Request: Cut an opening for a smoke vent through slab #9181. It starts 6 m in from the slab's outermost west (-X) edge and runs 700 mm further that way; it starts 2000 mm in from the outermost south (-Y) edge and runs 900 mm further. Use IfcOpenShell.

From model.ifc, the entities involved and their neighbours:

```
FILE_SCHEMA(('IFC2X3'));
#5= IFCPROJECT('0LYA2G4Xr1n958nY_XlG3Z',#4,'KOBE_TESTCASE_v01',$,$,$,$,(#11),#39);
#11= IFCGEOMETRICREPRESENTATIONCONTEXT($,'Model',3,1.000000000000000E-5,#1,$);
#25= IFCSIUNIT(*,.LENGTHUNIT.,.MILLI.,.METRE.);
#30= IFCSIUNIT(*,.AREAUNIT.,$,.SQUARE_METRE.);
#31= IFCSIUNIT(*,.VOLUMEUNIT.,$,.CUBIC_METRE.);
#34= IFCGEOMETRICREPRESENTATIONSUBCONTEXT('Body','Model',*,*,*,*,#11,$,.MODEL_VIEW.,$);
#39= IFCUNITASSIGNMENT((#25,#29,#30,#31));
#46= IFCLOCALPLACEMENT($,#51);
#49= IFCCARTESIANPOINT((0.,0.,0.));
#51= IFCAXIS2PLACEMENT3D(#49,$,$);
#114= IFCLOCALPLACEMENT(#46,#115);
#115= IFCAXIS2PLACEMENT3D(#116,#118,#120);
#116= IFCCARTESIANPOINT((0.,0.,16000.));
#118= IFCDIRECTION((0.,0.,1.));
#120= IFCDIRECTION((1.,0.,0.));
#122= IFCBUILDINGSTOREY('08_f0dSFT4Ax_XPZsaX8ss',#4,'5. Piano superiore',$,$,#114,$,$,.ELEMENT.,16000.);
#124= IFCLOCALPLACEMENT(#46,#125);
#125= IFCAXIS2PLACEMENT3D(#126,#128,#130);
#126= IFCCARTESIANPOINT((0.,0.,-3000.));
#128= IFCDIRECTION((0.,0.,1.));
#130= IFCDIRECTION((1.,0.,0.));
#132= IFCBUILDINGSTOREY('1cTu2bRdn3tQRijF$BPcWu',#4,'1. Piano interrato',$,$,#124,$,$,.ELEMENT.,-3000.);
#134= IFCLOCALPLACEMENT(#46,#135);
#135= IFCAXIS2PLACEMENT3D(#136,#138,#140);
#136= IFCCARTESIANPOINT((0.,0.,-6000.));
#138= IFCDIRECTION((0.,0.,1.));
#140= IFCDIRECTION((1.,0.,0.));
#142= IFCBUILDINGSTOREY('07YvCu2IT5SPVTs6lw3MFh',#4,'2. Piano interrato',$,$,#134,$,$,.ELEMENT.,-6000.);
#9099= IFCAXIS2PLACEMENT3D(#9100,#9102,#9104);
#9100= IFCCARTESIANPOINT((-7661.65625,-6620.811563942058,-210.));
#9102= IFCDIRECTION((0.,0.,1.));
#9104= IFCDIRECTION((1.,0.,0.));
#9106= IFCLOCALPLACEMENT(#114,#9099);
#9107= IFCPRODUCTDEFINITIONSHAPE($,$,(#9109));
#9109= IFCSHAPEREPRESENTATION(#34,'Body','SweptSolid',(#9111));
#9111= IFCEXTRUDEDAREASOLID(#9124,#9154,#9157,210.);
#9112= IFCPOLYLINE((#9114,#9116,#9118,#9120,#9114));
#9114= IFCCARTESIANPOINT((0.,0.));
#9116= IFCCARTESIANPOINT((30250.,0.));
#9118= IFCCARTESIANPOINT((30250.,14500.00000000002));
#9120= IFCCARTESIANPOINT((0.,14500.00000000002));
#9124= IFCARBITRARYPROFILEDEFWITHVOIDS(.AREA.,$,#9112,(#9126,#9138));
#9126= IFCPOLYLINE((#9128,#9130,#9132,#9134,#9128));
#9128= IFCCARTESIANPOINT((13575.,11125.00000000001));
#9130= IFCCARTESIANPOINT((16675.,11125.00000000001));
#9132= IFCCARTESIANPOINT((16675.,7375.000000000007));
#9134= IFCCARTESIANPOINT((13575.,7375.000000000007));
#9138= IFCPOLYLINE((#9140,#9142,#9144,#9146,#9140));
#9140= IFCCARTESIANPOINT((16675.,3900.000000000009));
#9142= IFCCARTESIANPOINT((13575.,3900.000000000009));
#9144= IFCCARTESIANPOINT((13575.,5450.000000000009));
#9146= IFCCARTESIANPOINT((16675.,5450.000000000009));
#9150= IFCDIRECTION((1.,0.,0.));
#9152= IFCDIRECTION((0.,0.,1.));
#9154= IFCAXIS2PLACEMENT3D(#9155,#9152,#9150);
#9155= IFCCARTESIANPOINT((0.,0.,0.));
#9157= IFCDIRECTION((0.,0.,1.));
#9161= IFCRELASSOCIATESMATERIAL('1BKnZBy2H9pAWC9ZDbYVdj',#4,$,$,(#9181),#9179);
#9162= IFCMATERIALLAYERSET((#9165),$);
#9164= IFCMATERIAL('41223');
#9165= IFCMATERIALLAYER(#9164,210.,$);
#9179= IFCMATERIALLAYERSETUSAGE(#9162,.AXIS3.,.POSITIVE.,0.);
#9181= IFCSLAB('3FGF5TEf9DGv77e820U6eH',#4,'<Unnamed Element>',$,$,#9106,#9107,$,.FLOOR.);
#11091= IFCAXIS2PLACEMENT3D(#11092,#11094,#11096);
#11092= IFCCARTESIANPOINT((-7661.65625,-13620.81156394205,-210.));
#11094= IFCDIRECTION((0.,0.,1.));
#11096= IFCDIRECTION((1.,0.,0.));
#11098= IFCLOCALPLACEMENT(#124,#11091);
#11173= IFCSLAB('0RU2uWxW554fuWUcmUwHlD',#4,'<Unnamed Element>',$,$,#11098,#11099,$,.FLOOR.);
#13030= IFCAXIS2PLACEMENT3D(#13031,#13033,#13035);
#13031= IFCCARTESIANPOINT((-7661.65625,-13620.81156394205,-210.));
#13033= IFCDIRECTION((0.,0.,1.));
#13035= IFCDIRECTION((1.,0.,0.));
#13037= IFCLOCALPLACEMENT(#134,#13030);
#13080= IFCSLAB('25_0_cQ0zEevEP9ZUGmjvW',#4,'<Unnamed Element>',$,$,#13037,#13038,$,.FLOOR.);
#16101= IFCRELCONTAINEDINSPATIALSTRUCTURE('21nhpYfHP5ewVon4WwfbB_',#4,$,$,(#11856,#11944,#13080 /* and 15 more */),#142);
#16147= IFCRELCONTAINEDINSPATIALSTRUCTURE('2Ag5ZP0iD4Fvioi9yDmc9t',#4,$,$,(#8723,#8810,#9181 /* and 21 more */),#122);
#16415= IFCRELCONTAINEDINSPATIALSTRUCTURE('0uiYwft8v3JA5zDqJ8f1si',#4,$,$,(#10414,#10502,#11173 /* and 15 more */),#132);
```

```python
import numpy as np
import ifcopenshell
import ifcopenshell.api.feature
import ifcopenshell.api.geometry
import ifcopenshell.api.root
import ifcopenshell.geom
import ifcopenshell.util.placement
import ifcopenshell.util.representation
import ifcopenshell.util.shape
import ifcopenshell.util.unit

model = ifcopenshell.open("model.ifc")
unit_scale = ifcopenshell.util.unit.calculate_unit_scale(model)
settings = ifcopenshell.geom.settings()


def volume(element):
    """Net volume in cubic metres, openings subtracted."""
    shape = ifcopenshell.geom.create_shape(settings, element)
    return ifcopenshell.util.shape.get_volume(shape.geometry)


slab = model.by_id(9181)
before = volume(slab)

# Extent in the slab's own axes, in metres. The edges named are its -X and -Y sides.
slab_shape = ifcopenshell.geom.create_shape(settings, slab)
vertices = ifcopenshell.util.shape.get_vertices(slab_shape.geometry)
x_min, y_min, bottom = vertices.min(axis=0)
top = vertices[:, 2].max()

opening = ifcopenshell.api.root.create_entity(model, ifc_class="IfcOpeningElement", name="Smoke vent opening")
context = ifcopenshell.util.representation.get_context(model, "Model", "Body", "MODEL_VIEW")
width, depth = 0.7, 0.9
outline = [(0.0, 0.0), (width, 0.0), (width, depth), (0.0, depth), (0.0, 0.0)]
# Overshoot both faces by 50 mm so the cut is clean.
shape = ifcopenshell.api.geometry.add_slab_representation(
    model, context=context, depth=top - bottom + 0.1, polyline=outline
)
ifcopenshell.api.geometry.assign_representation(model, product=opening, representation=shape)

matrix = ifcopenshell.util.placement.get_local_placement(slab.ObjectPlacement)
matrix[:, 3] = matrix @ np.append(np.array([x_min + 6, y_min + 2, bottom - 0.05]) / unit_scale, 1.0)
ifcopenshell.api.geometry.edit_object_placement(model, product=opening, matrix=matrix, is_si=False)
ifcopenshell.api.feature.add_feature(model, feature=opening, element=slab)

after = volume(slab)

print(f"slab volume {before:.3f} -> {after:.3f} m3")

model.write("model_rev.ifc")
```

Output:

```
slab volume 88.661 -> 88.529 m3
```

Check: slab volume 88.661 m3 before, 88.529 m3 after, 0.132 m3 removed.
